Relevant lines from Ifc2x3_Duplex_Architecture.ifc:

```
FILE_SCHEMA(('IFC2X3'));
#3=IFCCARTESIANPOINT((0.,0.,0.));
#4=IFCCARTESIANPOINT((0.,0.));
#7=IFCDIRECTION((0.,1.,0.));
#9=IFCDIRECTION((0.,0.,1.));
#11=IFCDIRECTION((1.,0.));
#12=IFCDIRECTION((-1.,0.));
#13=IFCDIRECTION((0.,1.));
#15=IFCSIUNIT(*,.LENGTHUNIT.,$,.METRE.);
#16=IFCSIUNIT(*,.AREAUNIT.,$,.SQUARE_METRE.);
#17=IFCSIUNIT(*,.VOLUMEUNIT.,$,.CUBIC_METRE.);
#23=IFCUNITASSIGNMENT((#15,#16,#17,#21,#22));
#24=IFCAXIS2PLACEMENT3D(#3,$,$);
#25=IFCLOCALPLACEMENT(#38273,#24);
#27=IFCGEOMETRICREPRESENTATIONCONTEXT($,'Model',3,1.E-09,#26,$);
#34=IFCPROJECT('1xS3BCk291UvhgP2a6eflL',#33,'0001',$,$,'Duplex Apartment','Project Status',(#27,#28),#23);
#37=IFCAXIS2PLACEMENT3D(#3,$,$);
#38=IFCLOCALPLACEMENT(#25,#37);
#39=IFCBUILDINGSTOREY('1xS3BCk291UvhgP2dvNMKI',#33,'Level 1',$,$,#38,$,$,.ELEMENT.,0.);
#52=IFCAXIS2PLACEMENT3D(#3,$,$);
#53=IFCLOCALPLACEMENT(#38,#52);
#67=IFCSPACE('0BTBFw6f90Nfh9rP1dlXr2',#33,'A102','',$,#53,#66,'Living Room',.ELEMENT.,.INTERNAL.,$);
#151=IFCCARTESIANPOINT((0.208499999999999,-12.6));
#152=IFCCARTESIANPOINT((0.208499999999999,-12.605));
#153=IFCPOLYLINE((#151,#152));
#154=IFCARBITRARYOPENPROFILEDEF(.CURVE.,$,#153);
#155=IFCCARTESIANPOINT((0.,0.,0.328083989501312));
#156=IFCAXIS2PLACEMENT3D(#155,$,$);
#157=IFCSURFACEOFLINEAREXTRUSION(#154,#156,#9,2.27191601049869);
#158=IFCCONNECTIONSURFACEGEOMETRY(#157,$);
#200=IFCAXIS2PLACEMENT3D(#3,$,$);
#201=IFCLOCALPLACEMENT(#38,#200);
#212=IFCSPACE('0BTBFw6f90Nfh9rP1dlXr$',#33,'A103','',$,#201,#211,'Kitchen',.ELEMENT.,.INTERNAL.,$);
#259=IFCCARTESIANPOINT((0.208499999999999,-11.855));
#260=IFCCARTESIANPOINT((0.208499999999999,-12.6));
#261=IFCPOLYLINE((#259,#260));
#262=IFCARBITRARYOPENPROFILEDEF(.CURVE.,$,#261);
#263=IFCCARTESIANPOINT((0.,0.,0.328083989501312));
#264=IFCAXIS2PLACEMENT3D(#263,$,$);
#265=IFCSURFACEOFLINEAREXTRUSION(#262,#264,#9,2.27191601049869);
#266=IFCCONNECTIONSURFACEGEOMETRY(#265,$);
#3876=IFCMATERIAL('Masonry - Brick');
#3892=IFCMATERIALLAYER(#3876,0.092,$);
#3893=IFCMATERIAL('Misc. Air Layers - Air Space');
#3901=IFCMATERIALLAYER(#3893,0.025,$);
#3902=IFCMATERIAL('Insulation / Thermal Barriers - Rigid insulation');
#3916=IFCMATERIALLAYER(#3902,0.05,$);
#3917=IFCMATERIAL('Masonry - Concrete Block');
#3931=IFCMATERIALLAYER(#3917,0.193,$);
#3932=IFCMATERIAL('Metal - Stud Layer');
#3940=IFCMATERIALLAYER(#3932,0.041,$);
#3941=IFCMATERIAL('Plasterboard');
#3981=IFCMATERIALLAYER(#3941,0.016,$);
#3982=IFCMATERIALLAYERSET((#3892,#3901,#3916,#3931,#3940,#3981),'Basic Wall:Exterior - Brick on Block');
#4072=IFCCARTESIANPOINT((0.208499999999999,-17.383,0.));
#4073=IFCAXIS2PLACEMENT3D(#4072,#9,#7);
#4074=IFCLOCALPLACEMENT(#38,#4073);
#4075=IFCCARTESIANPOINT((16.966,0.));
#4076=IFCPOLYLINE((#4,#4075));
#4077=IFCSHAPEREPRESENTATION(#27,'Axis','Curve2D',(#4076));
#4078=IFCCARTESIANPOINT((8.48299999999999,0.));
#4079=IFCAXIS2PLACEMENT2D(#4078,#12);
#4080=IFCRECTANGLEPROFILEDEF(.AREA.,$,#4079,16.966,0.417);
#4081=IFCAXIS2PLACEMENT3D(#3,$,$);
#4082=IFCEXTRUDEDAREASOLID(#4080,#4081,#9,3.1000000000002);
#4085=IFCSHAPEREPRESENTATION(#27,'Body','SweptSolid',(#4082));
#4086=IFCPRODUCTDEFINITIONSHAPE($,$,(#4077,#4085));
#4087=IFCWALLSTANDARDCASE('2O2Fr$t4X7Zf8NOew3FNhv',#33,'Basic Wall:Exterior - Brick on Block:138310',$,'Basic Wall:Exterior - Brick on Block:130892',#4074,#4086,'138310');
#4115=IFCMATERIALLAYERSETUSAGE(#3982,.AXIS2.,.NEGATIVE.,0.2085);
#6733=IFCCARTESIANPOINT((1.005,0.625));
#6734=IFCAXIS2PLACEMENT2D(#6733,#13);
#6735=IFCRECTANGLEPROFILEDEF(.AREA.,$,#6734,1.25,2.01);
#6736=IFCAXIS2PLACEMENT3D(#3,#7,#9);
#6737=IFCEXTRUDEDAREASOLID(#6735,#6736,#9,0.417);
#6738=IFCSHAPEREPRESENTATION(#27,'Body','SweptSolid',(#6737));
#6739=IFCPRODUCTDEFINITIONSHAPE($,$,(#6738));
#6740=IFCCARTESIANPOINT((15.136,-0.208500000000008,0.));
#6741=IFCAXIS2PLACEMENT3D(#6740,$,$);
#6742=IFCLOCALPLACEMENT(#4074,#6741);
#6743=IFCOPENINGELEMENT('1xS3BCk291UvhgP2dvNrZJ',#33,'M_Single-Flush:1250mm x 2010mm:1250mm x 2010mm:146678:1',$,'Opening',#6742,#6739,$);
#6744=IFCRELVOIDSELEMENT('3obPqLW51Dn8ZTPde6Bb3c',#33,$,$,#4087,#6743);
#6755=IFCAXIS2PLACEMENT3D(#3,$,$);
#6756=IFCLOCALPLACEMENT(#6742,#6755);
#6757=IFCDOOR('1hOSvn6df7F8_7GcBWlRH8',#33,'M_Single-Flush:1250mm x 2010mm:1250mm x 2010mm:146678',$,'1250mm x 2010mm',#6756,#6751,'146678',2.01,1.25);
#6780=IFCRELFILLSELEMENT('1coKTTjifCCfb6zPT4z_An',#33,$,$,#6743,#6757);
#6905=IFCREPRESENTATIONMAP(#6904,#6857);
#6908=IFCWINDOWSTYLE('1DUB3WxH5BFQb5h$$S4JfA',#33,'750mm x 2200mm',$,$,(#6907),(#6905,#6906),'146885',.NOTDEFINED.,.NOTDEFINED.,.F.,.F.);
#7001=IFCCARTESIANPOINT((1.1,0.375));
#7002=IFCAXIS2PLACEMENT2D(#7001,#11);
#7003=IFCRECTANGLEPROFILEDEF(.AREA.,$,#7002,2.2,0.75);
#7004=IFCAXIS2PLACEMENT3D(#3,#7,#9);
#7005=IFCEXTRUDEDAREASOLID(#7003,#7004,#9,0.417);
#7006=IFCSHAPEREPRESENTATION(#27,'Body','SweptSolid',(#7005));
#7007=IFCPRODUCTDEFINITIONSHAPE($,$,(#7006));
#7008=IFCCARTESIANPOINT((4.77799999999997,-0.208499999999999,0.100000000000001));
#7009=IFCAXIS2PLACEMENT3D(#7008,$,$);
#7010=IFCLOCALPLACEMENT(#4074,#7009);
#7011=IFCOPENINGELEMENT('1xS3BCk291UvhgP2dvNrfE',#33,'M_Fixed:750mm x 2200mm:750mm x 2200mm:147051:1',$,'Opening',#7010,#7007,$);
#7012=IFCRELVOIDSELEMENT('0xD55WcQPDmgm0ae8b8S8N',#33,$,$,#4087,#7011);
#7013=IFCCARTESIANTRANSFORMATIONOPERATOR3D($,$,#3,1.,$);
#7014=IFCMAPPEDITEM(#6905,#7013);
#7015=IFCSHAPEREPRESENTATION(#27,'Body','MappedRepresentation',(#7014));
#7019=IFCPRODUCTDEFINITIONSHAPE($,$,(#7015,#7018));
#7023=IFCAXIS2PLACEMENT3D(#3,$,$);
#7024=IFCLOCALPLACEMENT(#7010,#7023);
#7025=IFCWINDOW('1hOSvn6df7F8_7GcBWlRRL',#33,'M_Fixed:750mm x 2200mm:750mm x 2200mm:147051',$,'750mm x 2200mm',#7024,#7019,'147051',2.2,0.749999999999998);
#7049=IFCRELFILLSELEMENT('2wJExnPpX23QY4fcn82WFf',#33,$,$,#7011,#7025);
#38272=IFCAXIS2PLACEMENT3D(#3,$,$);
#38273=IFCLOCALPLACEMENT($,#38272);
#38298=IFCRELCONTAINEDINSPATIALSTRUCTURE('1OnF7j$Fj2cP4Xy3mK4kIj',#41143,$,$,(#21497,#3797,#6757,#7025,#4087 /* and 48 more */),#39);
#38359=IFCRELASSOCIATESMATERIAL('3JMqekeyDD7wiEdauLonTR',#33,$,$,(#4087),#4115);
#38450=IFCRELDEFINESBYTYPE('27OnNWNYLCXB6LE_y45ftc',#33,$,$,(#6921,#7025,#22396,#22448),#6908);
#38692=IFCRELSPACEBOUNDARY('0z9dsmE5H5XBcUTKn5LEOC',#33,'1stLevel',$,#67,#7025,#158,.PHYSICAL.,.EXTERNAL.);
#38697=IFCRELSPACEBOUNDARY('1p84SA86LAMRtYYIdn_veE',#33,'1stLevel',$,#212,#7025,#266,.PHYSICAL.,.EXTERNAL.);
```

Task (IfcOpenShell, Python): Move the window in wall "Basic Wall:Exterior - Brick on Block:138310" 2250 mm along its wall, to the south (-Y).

```python
import numpy as np
import ifcopenshell
import ifcopenshell.api.geometry
import ifcopenshell.util.placement
import ifcopenshell.util.unit

model = ifcopenshell.open("Ifc2x3_Duplex_Architecture.ifc")
unit_scale = ifcopenshell.util.unit.calculate_unit_scale(model)

window = model.by_guid("1hOSvn6df7F8_7GcBWlRRL")
opening = window.FillsVoids[0].RelatingOpeningElement
wall = opening.VoidsElements[0].RelatingBuildingElement

wall_matrix = ifcopenshell.util.placement.get_local_placement(wall.ObjectPlacement)
shift = wall_matrix[:3, 0] * -2.25 / unit_scale
before = ifcopenshell.util.placement.get_local_placement(window.ObjectPlacement)[:3, 3].copy()

# The window is placed relative to its opening, so it follows when the opening moves.
matrix = ifcopenshell.util.placement.get_local_placement(opening.ObjectPlacement)
matrix[:3, 3] += shift
ifcopenshell.api.geometry.edit_object_placement(
    model, product=opening, matrix=matrix, is_si=False, should_transform_children=True
)

# Space boundary surfaces are stored in each space's coordinates; move them too.
for rel in window.ProvidesBoundaries:
    if not rel.ConnectionGeometry:
        continue
    surface = rel.ConnectionGeometry.SurfaceOnRelatingElement
    space_matrix = ifcopenshell.util.placement.get_local_placement(rel.RelatingSpace.ObjectPlacement)
    point = np.array(surface.Position.Location.Coordinates) + space_matrix[:3, :3].T @ shift
    surface.Position = model.createIfcAxis2Placement3D(
        model.createIfcCartesianPoint(point.tolist()), surface.Position.Axis, surface.Position.RefDirection
    )

after = ifcopenshell.util.placement.get_local_placement(window.ObjectPlacement)[:3, 3]
print("window moved by", (after - before).round(3) + 0.0)

model.write("Ifc2x3_Duplex_Architecture_rev.ifc")
```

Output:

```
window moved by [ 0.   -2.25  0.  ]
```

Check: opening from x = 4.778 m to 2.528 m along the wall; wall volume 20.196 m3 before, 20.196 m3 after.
